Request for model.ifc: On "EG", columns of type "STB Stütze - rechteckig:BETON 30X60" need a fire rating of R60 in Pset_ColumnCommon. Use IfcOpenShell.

First a look at what the model holds.

```python
import ifcopenshell
import ifcopenshell.util.element

model = ifcopenshell.open("model.ifc")
print(model.schema)
storey = next(s for s in model.by_type("IfcBuildingStorey") if s.Name == "EG")
columns = [e for e in ifcopenshell.util.element.get_decomposition(storey) if e.is_a("IfcColumn")]
seen = {}
for e in columns:
    element_type = ifcopenshell.util.element.get_type(e)
    key = (element_type.Name if element_type != e and element_type else None, ifcopenshell.util.element.get_pset(e, "Pset_ColumnCommon", "FireRating"))
    seen[key] = seen.get(key, 0) + 1
for (name, value), count in sorted(seen.items(), key=str):
    print(count, "x", name, "|", value)
```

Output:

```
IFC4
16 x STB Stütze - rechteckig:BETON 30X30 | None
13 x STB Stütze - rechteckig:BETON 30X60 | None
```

```python
import ifcopenshell
import ifcopenshell.api.pset
import ifcopenshell.util.element

model = ifcopenshell.open("model.ifc")

storey = next(s for s in model.by_type("IfcBuildingStorey") if s.Name == "EG")
columns = [e for e in ifcopenshell.util.element.get_decomposition(storey) if e.is_a("IfcColumn")]

count = 0
for e in columns:
    element_type = ifcopenshell.util.element.get_type(e)
    if element_type in (None, e) or element_type.Name != "STB Stütze - rechteckig:BETON 30X60":
        continue
    # add_pset returns the element's existing set when there is one.
    pset = ifcopenshell.api.pset.add_pset(model, product=e, name="Pset_ColumnCommon")
    ifcopenshell.api.pset.edit_pset(model, pset=pset, properties={"FireRating": "R60"})
    count += 1

print(count, "columns updated")

model.write("model-out.ifc")
```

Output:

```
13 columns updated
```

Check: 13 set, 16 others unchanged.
